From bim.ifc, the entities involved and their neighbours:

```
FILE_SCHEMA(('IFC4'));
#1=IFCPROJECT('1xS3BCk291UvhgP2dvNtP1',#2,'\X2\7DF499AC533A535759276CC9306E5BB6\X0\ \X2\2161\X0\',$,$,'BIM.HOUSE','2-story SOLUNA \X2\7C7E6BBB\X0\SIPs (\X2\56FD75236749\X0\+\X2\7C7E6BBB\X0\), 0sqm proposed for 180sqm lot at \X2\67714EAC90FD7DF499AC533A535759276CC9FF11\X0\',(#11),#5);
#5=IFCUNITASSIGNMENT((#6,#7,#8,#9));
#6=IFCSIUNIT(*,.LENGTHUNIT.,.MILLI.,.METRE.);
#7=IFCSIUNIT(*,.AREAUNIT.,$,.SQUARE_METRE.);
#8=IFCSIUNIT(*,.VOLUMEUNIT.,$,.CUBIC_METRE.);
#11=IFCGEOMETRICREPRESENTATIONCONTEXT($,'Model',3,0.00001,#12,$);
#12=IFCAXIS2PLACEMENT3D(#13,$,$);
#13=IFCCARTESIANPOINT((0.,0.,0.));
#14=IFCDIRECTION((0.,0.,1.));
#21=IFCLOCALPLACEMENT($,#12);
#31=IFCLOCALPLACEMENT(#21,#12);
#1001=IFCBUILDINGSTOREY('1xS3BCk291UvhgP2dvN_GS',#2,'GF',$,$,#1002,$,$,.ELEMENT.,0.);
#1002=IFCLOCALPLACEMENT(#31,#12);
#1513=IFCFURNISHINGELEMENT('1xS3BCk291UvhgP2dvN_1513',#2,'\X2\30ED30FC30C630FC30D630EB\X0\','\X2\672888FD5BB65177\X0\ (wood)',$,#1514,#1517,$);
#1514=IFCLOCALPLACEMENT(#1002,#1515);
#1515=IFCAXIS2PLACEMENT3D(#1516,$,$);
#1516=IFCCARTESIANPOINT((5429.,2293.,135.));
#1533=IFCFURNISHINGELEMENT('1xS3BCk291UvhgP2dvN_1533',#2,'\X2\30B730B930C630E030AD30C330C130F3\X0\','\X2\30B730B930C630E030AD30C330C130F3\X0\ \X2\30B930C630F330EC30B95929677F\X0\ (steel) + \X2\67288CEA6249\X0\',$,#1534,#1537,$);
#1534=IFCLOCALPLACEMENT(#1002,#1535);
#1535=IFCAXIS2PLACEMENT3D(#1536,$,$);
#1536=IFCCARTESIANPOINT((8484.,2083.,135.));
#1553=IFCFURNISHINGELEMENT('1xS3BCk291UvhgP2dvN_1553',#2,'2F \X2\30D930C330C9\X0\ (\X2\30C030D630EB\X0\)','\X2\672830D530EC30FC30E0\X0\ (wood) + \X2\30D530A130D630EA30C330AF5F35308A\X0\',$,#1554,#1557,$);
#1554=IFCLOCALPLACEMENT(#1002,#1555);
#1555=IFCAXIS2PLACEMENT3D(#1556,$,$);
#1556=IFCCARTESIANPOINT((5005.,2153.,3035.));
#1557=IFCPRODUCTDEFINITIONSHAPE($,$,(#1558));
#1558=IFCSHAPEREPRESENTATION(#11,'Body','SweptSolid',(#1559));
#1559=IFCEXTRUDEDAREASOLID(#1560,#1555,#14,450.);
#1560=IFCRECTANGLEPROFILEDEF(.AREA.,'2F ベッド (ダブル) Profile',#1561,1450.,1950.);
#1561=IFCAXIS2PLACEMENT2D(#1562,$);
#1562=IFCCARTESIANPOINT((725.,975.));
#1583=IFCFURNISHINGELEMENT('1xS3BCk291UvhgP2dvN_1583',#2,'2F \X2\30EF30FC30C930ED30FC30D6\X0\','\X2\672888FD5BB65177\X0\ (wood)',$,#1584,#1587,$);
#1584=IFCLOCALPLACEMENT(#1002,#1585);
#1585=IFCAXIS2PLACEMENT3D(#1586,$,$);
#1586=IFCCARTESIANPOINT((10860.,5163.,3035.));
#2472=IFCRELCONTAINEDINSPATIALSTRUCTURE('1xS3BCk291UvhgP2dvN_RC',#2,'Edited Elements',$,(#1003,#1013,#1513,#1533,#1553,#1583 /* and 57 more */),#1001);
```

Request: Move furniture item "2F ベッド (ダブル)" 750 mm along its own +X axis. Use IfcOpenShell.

```python
import ifcopenshell
import ifcopenshell.api.geometry
import ifcopenshell.util.placement

model = ifcopenshell.open("bim.ifc")

item = model.by_id(1553)
matrix = ifcopenshell.util.placement.get_local_placement(item.ObjectPlacement)
matrix[:3, 3] += matrix[:3, 0] * 750.0
ifcopenshell.api.geometry.edit_object_placement(model, product=item, matrix=matrix, is_si=False)

print(ifcopenshell.util.placement.get_local_placement(item.ObjectPlacement).round(3) + 0.0)

model.write("bim_v2.ifc")
```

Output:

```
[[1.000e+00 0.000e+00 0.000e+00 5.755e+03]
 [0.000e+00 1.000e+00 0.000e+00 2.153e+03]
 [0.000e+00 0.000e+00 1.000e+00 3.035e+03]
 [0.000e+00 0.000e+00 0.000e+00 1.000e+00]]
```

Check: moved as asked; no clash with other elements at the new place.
